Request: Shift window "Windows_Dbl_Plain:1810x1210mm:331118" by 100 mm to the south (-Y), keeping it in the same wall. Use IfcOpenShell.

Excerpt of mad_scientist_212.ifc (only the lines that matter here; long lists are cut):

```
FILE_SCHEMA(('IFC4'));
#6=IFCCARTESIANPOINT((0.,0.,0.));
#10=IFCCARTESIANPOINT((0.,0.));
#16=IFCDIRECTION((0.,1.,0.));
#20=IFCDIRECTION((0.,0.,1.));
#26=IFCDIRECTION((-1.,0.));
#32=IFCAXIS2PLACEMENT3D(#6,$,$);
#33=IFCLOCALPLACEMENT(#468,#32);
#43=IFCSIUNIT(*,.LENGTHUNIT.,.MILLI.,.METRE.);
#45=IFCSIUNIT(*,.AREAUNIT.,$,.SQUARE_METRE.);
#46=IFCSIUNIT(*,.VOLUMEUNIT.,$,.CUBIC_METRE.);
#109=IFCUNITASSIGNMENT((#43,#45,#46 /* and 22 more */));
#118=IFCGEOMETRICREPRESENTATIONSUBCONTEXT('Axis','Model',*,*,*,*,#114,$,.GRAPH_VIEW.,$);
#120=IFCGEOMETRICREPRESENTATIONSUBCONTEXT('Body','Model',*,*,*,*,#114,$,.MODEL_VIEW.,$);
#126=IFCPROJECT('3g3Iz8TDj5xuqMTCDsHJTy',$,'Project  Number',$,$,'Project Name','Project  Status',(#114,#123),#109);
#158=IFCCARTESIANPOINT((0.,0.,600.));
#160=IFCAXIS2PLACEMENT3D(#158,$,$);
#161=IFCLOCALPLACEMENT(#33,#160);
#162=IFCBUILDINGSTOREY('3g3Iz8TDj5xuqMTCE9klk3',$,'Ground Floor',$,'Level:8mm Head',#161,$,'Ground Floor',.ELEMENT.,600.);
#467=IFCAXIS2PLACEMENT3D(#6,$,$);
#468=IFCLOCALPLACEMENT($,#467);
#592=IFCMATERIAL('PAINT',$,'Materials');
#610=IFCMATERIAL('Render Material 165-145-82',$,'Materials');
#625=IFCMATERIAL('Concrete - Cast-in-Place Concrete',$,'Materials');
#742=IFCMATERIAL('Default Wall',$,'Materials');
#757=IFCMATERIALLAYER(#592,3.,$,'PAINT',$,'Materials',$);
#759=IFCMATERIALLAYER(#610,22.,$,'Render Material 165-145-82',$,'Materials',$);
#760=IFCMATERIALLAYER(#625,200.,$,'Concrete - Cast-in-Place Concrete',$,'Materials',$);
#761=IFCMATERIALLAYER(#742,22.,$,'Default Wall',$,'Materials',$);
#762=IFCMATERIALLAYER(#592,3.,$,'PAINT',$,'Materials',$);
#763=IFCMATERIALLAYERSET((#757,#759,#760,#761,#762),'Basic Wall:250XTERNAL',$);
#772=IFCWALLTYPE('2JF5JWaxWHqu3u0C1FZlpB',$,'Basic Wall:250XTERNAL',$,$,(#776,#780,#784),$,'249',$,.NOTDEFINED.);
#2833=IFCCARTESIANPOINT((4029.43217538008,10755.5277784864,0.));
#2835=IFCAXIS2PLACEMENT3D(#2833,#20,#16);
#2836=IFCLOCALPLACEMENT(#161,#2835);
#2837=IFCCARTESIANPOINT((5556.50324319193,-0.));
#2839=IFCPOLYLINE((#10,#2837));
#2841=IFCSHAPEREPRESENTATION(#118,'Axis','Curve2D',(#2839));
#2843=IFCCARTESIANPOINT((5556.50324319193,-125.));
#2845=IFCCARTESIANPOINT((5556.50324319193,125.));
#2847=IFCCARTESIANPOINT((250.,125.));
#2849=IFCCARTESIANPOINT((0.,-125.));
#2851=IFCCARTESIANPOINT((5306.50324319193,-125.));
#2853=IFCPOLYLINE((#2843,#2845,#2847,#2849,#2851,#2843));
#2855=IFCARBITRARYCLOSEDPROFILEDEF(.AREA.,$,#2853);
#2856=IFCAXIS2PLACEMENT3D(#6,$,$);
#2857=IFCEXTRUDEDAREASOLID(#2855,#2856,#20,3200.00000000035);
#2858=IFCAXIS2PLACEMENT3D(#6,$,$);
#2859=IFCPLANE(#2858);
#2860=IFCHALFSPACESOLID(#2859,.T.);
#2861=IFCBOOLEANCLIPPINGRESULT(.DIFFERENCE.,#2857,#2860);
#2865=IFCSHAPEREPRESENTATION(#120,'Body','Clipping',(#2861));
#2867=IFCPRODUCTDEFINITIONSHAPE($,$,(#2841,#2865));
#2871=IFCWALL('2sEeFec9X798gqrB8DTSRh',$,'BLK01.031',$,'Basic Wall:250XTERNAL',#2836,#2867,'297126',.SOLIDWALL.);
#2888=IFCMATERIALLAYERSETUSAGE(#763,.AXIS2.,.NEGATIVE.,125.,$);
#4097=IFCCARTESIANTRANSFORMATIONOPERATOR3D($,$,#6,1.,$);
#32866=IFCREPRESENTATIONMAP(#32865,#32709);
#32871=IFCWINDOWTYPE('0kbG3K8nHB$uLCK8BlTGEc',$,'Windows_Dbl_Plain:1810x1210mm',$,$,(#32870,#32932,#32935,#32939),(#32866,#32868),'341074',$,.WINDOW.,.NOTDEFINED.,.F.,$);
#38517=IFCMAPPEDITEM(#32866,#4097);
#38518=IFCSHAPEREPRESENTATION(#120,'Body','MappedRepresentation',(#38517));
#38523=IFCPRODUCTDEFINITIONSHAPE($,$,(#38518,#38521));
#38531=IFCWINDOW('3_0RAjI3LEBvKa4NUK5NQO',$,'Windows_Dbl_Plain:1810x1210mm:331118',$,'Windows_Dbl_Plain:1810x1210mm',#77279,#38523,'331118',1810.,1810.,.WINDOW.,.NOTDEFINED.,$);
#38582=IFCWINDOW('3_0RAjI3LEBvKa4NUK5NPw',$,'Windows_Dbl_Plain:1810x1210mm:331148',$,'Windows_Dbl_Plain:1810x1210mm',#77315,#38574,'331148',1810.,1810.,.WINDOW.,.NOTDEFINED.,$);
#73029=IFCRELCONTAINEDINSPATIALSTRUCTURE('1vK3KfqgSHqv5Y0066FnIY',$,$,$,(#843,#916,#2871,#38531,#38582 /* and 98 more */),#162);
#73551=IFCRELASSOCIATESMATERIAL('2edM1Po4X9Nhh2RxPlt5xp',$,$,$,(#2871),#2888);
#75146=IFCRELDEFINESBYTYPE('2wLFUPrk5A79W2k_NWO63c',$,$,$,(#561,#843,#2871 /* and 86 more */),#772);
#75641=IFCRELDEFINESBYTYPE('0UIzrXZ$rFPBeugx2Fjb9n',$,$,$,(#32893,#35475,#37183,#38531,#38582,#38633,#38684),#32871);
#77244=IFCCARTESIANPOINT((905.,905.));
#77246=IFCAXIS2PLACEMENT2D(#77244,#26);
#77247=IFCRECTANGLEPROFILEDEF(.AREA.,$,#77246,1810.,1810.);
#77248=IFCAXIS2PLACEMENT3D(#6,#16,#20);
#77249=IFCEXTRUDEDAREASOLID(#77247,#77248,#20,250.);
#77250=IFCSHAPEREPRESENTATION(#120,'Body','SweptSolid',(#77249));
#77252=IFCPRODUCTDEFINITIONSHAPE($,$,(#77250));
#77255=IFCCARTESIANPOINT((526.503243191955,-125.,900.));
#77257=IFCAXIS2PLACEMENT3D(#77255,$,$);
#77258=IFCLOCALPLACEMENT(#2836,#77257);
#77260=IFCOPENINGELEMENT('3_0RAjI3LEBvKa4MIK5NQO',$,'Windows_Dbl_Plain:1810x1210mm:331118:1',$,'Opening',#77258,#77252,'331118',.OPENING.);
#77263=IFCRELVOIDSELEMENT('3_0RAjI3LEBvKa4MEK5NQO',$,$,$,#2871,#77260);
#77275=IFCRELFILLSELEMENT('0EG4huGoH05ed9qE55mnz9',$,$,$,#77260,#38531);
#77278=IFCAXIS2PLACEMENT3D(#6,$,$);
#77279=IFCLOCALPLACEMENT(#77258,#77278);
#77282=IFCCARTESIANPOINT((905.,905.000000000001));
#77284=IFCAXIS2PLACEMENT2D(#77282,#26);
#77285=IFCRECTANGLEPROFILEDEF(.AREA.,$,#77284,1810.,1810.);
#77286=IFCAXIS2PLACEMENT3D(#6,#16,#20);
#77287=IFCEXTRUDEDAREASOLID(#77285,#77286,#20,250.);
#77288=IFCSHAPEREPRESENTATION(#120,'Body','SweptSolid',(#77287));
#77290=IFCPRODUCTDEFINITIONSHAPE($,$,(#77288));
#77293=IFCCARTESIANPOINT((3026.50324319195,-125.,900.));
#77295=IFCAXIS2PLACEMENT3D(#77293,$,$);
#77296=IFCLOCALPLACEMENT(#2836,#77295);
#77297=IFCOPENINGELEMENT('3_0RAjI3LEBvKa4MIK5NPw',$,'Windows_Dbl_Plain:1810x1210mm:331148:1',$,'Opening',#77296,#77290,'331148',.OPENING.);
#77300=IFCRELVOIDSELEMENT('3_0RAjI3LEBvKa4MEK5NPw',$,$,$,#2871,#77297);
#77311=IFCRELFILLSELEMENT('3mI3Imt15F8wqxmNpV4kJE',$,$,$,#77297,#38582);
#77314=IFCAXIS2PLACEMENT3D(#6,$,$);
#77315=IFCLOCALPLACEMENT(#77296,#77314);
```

```python
import ifcopenshell
import ifcopenshell.api.geometry
import ifcopenshell.util.placement
import ifcopenshell.util.unit

model = ifcopenshell.open("mad_scientist_212.ifc")
unit_scale = ifcopenshell.util.unit.calculate_unit_scale(model)

window = model.by_id(38531)
opening = window.FillsVoids[0].RelatingOpeningElement
wall = opening.VoidsElements[0].RelatingBuildingElement

wall_matrix = ifcopenshell.util.placement.get_local_placement(wall.ObjectPlacement)
shift = wall_matrix[:3, 0] * -0.1 / unit_scale
before = ifcopenshell.util.placement.get_local_placement(window.ObjectPlacement)[:3, 3].copy()

# The window is placed relative to its opening, so it follows when the opening moves.
matrix = ifcopenshell.util.placement.get_local_placement(opening.ObjectPlacement)
matrix[:3, 3] += shift
ifcopenshell.api.geometry.edit_object_placement(
    model, product=opening, matrix=matrix, is_si=False, should_transform_children=True
)

after = ifcopenshell.util.placement.get_local_placement(window.ObjectPlacement)[:3, 3]
print("window moved by", (after - before).round(3) + 0.0)

model.write("mad_scientist_212_rev.ifc")
```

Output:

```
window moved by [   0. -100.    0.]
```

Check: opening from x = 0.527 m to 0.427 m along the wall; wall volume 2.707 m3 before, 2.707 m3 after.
